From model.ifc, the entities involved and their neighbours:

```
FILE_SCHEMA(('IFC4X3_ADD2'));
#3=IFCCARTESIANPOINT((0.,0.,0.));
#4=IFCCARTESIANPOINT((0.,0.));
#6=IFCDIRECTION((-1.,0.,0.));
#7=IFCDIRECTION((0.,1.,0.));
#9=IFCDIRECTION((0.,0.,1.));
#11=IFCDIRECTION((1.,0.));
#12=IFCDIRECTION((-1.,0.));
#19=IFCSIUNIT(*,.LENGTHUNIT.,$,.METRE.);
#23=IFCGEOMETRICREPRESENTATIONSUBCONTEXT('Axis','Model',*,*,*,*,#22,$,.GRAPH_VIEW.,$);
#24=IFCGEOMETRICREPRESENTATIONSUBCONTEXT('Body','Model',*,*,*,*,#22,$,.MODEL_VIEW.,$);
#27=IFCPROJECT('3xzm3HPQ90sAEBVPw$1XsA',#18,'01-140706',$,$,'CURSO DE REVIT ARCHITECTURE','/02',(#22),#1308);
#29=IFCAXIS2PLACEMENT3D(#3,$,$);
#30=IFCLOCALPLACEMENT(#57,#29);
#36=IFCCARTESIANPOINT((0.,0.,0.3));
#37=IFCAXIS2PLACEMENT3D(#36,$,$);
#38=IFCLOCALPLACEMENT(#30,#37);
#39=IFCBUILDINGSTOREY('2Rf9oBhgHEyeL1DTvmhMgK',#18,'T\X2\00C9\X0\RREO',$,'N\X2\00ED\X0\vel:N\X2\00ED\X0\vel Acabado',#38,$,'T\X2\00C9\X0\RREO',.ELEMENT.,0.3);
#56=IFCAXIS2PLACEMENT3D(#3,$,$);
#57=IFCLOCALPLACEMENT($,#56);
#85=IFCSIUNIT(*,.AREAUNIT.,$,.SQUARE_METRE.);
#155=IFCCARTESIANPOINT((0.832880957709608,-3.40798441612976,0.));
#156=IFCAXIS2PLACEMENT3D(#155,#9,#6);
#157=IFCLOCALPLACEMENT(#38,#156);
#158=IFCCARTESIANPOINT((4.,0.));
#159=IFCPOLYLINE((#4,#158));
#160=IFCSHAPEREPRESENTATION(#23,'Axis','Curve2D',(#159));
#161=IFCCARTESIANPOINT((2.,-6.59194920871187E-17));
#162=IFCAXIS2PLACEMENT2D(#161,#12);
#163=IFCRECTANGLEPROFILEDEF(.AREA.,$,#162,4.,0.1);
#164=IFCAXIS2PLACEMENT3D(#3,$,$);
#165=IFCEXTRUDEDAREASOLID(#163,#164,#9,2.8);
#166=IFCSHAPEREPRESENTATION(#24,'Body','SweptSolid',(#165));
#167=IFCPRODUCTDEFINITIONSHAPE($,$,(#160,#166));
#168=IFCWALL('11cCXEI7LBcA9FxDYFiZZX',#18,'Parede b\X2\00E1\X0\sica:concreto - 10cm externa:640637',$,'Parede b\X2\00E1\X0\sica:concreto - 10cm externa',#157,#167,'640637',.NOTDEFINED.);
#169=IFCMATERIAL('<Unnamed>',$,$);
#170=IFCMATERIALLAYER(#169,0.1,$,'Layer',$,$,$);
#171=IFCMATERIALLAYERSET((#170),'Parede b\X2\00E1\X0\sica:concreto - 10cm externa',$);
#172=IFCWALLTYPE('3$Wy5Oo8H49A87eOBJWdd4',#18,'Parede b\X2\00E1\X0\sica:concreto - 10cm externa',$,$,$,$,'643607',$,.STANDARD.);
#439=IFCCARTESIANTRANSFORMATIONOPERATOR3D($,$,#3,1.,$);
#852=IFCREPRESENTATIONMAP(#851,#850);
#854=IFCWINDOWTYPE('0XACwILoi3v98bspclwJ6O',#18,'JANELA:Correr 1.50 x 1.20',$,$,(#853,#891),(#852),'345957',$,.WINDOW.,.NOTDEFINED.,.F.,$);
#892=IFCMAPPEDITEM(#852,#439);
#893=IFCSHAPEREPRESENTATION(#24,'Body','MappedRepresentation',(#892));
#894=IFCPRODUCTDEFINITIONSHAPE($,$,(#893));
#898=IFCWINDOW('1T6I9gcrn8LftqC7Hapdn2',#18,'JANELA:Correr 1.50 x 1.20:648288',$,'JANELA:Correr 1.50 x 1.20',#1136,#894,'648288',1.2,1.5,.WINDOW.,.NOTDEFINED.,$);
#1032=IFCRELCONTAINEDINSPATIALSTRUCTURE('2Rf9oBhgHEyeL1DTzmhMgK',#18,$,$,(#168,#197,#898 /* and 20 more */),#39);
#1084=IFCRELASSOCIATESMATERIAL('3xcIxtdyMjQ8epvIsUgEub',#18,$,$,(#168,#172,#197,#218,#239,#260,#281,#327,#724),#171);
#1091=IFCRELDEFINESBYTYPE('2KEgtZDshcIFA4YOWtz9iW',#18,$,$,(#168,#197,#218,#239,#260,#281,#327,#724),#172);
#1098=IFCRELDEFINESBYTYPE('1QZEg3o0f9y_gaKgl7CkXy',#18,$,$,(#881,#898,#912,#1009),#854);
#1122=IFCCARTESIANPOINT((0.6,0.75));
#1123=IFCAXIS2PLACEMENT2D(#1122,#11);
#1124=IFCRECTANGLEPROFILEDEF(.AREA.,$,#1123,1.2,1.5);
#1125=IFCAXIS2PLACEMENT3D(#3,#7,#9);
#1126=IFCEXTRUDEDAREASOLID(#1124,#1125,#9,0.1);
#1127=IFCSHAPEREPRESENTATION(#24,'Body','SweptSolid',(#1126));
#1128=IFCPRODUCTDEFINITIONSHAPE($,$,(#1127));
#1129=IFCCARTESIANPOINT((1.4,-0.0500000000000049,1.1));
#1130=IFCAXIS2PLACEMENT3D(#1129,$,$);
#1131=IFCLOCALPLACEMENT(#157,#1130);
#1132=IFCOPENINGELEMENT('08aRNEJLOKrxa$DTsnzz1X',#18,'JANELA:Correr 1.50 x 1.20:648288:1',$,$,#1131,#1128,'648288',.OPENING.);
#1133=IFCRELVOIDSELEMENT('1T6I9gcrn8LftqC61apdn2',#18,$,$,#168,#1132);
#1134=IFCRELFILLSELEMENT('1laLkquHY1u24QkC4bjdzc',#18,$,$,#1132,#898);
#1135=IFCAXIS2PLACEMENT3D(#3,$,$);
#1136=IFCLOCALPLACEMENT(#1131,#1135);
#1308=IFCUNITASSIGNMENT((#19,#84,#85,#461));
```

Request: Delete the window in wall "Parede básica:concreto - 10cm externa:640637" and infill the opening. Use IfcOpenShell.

```python
import ifcopenshell
import ifcopenshell.api.feature
import ifcopenshell.api.root
import ifcopenshell.geom
import ifcopenshell.util.shape

model = ifcopenshell.open("model.ifc")
settings = ifcopenshell.geom.settings()


def volume(element):
    """Net volume in cubic metres, openings subtracted."""
    shape = ifcopenshell.geom.create_shape(settings, element)
    return ifcopenshell.util.shape.get_volume(shape.geometry)


window = model.by_guid("1T6I9gcrn8LftqC7Hapdn2")
opening = window.FillsVoids[0].RelatingOpeningElement
wall = opening.VoidsElements[0].RelatingBuildingElement
before = volume(wall)

ifcopenshell.api.root.remove_product(model, product=window)
ifcopenshell.api.feature.remove_feature(model, feature=opening)

after = volume(wall)

print(f"wall volume {before:.3f} -> {after:.3f} m3")

model.write("model_v2.ifc")
```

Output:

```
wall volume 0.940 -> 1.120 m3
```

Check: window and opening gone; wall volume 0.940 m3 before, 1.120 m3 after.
